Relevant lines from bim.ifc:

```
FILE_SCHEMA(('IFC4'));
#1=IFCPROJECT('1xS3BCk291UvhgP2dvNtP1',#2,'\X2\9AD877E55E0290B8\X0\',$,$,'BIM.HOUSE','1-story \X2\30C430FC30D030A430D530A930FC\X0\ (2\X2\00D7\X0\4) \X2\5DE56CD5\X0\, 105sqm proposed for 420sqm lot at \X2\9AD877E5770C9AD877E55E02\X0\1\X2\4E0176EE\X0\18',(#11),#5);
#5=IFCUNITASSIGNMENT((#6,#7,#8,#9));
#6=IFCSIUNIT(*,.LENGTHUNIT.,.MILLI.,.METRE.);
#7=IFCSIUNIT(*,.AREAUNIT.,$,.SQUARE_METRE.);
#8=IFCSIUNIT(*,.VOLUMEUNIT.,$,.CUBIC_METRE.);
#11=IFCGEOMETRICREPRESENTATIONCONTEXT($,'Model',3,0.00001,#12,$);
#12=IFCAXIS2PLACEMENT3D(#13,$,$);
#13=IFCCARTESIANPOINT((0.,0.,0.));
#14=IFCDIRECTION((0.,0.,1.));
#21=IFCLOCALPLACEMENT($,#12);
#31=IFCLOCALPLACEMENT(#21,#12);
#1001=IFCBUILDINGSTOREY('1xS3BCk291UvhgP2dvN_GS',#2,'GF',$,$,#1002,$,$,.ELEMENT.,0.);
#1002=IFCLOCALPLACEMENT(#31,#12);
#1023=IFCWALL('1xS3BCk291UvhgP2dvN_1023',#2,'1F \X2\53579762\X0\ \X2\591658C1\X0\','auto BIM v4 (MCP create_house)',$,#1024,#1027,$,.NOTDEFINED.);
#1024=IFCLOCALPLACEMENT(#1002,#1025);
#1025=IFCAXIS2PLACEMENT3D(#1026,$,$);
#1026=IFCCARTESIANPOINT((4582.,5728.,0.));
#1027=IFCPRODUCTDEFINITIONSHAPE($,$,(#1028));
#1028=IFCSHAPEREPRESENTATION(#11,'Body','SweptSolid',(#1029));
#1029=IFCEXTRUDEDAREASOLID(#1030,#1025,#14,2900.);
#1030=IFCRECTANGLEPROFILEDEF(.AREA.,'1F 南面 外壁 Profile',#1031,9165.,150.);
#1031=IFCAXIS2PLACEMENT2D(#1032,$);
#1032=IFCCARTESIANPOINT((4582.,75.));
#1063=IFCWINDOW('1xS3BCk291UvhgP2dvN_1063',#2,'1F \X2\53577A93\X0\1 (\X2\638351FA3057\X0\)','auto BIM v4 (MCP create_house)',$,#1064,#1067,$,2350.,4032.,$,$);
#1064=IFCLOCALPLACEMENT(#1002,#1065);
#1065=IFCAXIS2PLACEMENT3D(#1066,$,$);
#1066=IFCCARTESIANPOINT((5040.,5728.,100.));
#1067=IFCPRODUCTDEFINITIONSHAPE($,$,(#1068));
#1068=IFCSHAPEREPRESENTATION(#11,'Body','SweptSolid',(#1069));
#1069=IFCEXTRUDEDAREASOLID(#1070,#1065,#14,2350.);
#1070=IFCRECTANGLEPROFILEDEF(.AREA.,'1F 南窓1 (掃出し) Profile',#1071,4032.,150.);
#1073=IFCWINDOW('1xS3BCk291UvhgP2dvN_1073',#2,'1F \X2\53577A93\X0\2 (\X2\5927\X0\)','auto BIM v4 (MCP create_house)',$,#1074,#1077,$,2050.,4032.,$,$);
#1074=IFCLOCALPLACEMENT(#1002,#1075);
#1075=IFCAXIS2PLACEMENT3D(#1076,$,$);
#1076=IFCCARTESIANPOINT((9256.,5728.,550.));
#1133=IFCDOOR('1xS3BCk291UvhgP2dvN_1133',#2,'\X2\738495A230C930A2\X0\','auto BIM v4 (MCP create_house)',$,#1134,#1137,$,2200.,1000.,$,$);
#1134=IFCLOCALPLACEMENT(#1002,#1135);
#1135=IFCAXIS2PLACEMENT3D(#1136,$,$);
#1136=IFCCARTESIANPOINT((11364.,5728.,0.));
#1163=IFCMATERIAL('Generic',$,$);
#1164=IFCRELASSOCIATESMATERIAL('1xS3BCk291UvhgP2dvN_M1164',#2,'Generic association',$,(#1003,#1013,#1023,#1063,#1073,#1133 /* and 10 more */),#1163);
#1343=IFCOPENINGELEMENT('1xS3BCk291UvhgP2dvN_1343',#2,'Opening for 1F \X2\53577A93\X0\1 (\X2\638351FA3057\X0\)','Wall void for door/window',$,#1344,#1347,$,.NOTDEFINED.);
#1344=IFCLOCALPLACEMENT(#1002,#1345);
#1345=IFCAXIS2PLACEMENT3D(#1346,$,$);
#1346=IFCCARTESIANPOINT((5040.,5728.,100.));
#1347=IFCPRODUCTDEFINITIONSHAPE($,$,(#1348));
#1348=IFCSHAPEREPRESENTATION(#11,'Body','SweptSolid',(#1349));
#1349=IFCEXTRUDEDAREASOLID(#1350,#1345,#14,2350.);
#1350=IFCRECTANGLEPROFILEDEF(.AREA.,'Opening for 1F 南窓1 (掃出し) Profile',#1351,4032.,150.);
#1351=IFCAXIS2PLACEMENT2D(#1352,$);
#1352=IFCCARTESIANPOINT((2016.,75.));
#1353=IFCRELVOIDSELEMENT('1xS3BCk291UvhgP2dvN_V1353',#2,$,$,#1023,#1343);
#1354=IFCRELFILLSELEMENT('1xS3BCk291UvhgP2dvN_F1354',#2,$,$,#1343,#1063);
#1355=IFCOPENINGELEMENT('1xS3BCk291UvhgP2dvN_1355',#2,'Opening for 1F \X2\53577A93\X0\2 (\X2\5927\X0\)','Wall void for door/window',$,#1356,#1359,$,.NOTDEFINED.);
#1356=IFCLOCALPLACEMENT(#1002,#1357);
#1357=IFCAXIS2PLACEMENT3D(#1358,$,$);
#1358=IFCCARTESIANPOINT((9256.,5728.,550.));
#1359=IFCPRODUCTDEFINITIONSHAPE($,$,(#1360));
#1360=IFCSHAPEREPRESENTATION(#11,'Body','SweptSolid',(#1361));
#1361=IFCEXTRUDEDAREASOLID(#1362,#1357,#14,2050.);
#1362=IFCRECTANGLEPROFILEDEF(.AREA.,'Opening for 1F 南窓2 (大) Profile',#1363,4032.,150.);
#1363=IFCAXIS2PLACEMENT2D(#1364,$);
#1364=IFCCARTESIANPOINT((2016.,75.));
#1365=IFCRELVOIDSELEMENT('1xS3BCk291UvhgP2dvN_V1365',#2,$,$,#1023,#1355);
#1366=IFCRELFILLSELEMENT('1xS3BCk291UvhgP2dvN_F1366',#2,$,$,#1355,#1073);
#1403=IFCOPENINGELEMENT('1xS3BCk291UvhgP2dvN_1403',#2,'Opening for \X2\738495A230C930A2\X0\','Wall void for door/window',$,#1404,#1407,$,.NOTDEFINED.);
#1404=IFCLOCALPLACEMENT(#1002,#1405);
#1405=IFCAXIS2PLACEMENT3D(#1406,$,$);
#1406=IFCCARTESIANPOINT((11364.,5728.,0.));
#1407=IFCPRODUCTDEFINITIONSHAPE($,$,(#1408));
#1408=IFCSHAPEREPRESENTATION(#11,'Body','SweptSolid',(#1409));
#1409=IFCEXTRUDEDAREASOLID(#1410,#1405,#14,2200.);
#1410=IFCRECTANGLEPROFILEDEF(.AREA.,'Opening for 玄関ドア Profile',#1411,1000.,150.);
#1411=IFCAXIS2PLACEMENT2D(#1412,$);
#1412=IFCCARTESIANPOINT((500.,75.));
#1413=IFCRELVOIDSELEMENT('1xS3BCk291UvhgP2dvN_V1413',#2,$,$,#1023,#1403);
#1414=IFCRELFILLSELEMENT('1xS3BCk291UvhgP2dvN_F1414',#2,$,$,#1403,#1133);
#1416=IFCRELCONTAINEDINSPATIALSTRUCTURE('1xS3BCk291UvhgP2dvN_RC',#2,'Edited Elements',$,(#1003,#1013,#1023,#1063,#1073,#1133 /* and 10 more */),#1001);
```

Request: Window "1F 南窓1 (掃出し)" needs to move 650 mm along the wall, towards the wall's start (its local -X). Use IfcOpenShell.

```python
import ifcopenshell
import ifcopenshell.api.geometry
import ifcopenshell.util.placement

model = ifcopenshell.open("bim.ifc")

window = model.by_guid("1xS3BCk291UvhgP2dvN_1063")
opening = window.FillsVoids[0].RelatingOpeningElement
wall = opening.VoidsElements[0].RelatingBuildingElement

wall_matrix = ifcopenshell.util.placement.get_local_placement(wall.ObjectPlacement)
shift = wall_matrix[:3, 0] * -650.0
before = ifcopenshell.util.placement.get_local_placement(window.ObjectPlacement)[:3, 3].copy()

# The window is not placed relative to its opening, so move both.
for product in (opening, window):
    matrix = ifcopenshell.util.placement.get_local_placement(product.ObjectPlacement)
    matrix[:3, 3] += shift
    ifcopenshell.api.geometry.edit_object_placement(model, product=product, matrix=matrix, is_si=False)

after = ifcopenshell.util.placement.get_local_placement(window.ObjectPlacement)[:3, 3]
print("window moved by", (after - before).round(3) + 0.0)

model.write("bim_rev.ifc")
```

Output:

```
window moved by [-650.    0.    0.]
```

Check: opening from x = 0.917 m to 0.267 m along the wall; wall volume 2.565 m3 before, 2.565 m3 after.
